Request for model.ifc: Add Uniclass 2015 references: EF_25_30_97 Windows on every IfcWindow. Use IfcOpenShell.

First a look at what the model holds.

```python
import ifcopenshell

model = ifcopenshell.open("model.ifc")
print(model.schema)
print("classifications:", [c.Name for c in model.by_type("IfcClassification")])
for ifc_class in ("IfcDoor", "IfcRoof", "IfcStair", "IfcWall", "IfcWindow"):
    print(ifc_class, len(model.by_type(ifc_class)))
```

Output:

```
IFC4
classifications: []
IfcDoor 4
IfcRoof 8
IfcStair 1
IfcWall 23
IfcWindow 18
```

```python
import ifcopenshell
import ifcopenshell.api.classification

model = ifcopenshell.open("model.ifc")

system = ifcopenshell.api.classification.add_classification(model, classification="Uniclass 2015")

codes = {
    "IfcWindow": ("EF_25_30_97", "Windows"),
}
for ifc_class, (code, name) in codes.items():
    products = model.by_type(ifc_class)
    ifcopenshell.api.classification.add_reference(
        model, products=products, classification=system, identification=code, name=name
    )
    print(code, len(products))

model.write("model_updated.ifc")
```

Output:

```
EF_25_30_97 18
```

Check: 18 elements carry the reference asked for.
